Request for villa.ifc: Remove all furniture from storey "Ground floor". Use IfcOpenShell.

First a look at what the model holds.

```python
import ifcopenshell
import ifcopenshell.util.element

model = ifcopenshell.open("villa.ifc")
print(model.schema)
storey = next(s for s in model.by_type("IfcBuildingStorey") if s.Name == "Ground floor")
furniture = [e for e in ifcopenshell.util.element.get_decomposition(storey) if e.is_a("IfcFurnishingElement")]
seen = {}
for e in furniture:
    element_type = ifcopenshell.util.element.get_type(e)
    name = element_type.Name if element_type not in (None, e) else None
    seen[name] = seen.get(name, 0) + 1
for name, count in sorted(seen.items(), key=str):
    print(count, "x", name)
```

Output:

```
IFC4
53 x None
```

```python
import ifcopenshell
import ifcopenshell.api.root
import ifcopenshell.util.element

model = ifcopenshell.open("villa.ifc")

storey = next(s for s in model.by_type("IfcBuildingStorey") if s.Name == "Ground floor")
furniture = [e for e in ifcopenshell.util.element.get_decomposition(storey) if e.is_a("IfcFurnishingElement")]

for e in furniture:
    ifcopenshell.api.root.remove_product(model, product=e)
print(len(furniture), "removed")

model.write("villa_edited.ifc")
```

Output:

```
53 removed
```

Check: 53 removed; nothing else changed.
